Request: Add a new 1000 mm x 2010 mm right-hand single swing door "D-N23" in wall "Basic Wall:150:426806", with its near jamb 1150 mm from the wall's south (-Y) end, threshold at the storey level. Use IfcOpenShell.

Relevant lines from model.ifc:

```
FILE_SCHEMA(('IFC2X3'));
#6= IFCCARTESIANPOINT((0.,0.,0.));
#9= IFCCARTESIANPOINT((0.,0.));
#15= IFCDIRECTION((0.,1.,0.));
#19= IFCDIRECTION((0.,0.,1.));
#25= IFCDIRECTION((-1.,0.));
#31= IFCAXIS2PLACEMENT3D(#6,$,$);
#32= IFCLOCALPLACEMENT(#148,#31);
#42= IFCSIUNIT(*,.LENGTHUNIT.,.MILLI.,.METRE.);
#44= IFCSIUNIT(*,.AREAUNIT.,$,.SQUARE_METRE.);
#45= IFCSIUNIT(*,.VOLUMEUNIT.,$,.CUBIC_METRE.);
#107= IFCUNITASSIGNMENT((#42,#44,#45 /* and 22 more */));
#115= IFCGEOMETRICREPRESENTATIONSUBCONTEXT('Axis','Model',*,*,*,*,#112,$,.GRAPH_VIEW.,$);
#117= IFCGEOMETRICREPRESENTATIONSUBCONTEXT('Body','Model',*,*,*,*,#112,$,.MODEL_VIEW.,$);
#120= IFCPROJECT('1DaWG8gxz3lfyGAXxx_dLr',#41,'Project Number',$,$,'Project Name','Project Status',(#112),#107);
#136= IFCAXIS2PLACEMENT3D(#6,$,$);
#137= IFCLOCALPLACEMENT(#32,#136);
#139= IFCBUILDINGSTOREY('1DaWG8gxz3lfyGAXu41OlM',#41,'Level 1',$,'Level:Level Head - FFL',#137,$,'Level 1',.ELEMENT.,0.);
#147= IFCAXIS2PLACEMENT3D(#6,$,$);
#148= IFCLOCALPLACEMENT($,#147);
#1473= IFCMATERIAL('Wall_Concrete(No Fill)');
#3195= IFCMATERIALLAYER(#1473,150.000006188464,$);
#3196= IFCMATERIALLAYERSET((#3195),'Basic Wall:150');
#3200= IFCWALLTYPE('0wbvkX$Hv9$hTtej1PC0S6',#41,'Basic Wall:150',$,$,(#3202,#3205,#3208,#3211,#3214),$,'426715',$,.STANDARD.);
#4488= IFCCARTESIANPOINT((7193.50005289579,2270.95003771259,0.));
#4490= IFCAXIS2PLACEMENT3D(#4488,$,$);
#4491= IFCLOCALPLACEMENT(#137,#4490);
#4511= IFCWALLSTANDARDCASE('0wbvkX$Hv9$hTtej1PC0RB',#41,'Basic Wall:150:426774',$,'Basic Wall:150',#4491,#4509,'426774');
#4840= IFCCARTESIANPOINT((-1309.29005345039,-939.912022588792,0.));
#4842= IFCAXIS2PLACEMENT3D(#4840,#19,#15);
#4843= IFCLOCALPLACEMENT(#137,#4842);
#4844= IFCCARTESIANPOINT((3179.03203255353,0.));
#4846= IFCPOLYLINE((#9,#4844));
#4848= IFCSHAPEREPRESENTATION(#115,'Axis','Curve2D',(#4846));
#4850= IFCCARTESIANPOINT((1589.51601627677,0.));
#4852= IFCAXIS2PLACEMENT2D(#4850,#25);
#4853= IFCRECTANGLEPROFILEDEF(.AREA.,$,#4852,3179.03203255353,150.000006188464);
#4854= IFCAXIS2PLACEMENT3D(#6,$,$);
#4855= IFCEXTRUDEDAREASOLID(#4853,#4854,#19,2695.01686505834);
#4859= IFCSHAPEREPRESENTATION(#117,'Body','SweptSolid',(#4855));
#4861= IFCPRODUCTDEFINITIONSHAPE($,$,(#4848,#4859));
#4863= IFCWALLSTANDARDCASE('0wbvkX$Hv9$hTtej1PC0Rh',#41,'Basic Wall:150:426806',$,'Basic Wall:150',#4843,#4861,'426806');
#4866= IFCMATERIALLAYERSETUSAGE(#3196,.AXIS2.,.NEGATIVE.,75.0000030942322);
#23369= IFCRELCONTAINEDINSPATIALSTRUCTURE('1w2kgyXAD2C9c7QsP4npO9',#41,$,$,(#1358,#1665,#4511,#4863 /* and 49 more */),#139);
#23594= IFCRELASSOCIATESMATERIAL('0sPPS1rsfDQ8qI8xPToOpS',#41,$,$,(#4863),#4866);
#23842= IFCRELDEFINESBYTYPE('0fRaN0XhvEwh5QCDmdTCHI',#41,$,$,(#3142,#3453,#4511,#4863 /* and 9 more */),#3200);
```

```python
import numpy as np
import ifcopenshell
import ifcopenshell.api.feature
import ifcopenshell.api.geometry
import ifcopenshell.api.root
import ifcopenshell.api.spatial
import ifcopenshell.api.type
import ifcopenshell.geom
import ifcopenshell.util.element
import ifcopenshell.util.placement
import ifcopenshell.util.representation
import ifcopenshell.util.shape
import ifcopenshell.util.unit

model = ifcopenshell.open("model.ifc")
unit_scale = ifcopenshell.util.unit.calculate_unit_scale(model)
settings = ifcopenshell.geom.settings()


def volume(element):
    """Net volume in cubic metres, openings subtracted."""
    shape = ifcopenshell.geom.create_shape(settings, element)
    return ifcopenshell.util.shape.get_volume(shape.geometry)


wall = model.by_guid("0wbvkX$Hv9$hTtej1PC0Rh")
storey = ifcopenshell.util.element.get_container(wall, ifc_class="IfcBuildingStorey")
context = ifcopenshell.util.representation.get_context(model, "Model", "Body", "MODEL_VIEW")
before = volume(wall)

width, height, from_end, sill = 1, 2.01, 1.15, 0.0  # metres

# The wall runs along its own X axis, and the end named is its -X end.
wall_shape = ifcopenshell.geom.create_shape(settings, wall)
x, y, z = ifcopenshell.util.shape.get_vertices(wall_shape.geometry).T
start = x.min() + from_end
face, thickness = float(y.min()), float(y.max() - y.min())
wall_matrix = ifcopenshell.util.placement.get_local_placement(wall.ObjectPlacement)
level = ifcopenshell.util.placement.get_local_placement(storey.ObjectPlacement)[2, 3]


def in_wall(x, y):
    """Placement at x, y metres in the wall's axes, at sill height."""
    matrix = wall_matrix.copy()
    matrix[:, 3] = wall_matrix @ np.array([x / unit_scale, y / unit_scale, 0.0, 1.0])
    matrix[2, 3] = level + sill / unit_scale
    return matrix


# Opening: a box that overshoots both wall faces by 50 mm.
opening = ifcopenshell.api.root.create_entity(model, ifc_class="IfcOpeningElement")
box = ifcopenshell.api.geometry.add_wall_representation(
    model, context=context, length=width, height=height, thickness=thickness + 0.1
)
ifcopenshell.api.geometry.assign_representation(model, product=opening, representation=box)
ifcopenshell.api.geometry.edit_object_placement(model, product=opening, matrix=in_wall(start, face - 0.05), is_si=False)
ifcopenshell.api.feature.add_feature(model, feature=opening, element=wall)

door = ifcopenshell.api.root.create_entity(model, ifc_class="IfcDoor", name="D-N23")
door.OverallWidth, door.OverallHeight = width / unit_scale, height / unit_scale
body = ifcopenshell.api.geometry.add_door_representation(
    model,
    context=context,
    overall_width=door.OverallWidth,
    overall_height=door.OverallHeight,
    operation_type="SINGLE_SWING_RIGHT",
    lining_properties={"LiningDepth": thickness / unit_scale, "ThresholdDepth": thickness / unit_scale},
)
ifcopenshell.api.geometry.assign_representation(model, product=door, representation=body)
ifcopenshell.api.spatial.assign_container(model, products=[door], relating_structure=storey)
fills = ifcopenshell.api.feature.add_filling(model, opening=opening, element=door)
fills.OwnerHistory = door.OwnerHistory  # required in IFC2X3

# IFC2X3 keeps the operation on the door style.
style = ifcopenshell.api.root.create_entity(model, ifc_class="IfcDoorStyle", name="D-N23")
style.OperationType, style.ConstructionType = "SINGLE_SWING_RIGHT", "NOTDEFINED"
style.ParameterTakesPrecedence = style.Sizeable = False
ifcopenshell.api.type.assign_type(model, related_objects=[door], relating_type=style)

# The lining spans the wall, so the door starts at the wall face.
ifcopenshell.api.geometry.edit_object_placement(model, product=door, matrix=in_wall(start, face), is_si=False)

after = volume(wall)

print(f"wall volume {before:.3f} -> {after:.3f} m3")

model.write("model_edited.ifc")
```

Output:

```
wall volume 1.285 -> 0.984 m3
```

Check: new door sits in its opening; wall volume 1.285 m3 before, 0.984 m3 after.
